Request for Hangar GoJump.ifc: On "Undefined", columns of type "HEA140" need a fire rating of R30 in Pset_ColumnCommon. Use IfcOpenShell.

First a look at what the model holds.

```python
import ifcopenshell
import ifcopenshell.util.element

model = ifcopenshell.open("Hangar GoJump.ifc")
print(model.schema)
storey = next(s for s in model.by_type("IfcBuildingStorey") if s.Name == "Undefined")
columns = [e for e in ifcopenshell.util.element.get_decomposition(storey) if e.is_a("IfcColumn")]
seen = {}
for e in columns:
    element_type = ifcopenshell.util.element.get_type(e)
    key = (element_type.Name if element_type != e and element_type else None, ifcopenshell.util.element.get_pset(e, "Pset_ColumnCommon", "FireRating"))
    seen[key] = seen.get(key, 0) + 1
for (name, value), count in sorted(seen.items(), key=str):
    print(count, "x", name, "|", value)
```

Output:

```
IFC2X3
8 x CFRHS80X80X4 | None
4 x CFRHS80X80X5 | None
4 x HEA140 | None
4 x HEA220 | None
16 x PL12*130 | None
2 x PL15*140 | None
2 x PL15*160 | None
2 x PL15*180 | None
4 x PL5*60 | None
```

```python
import ifcopenshell
import ifcopenshell.api.pset
import ifcopenshell.util.element

model = ifcopenshell.open("Hangar GoJump.ifc")

storey = next(s for s in model.by_type("IfcBuildingStorey") if s.Name == "Undefined")
columns = [e for e in ifcopenshell.util.element.get_decomposition(storey) if e.is_a("IfcColumn")]

count = 0
for e in columns:
    element_type = ifcopenshell.util.element.get_type(e)
    if element_type in (None, e) or element_type.Name != "HEA140":
        continue
    # add_pset returns the element's existing set when there is one.
    pset = ifcopenshell.api.pset.add_pset(model, product=e, name="Pset_ColumnCommon")
    ifcopenshell.api.pset.edit_pset(model, pset=pset, properties={"FireRating": "R30"})
    count += 1

print(count, "columns updated")

model.write("Hangar GoJump-out.ifc")
```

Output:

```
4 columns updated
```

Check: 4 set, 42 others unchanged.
